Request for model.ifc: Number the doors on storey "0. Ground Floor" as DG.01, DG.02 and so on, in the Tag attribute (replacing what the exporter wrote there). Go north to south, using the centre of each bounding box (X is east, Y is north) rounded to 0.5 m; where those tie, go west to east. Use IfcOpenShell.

First a look at what the model holds.

```python
import ifcopenshell
import ifcopenshell.util.element
import ifcopenshell.util.placement

model = ifcopenshell.open("model.ifc")
print(model.schema)
storey = next(s for s in model.by_type("IfcBuildingStorey") if s.Name == "0. Ground Floor")
doors = [e for e in ifcopenshell.util.element.get_decomposition(storey) if e.is_a("IfcDoor")]
for e in sorted(doors, key=lambda e: e.id()):
    origin = ifcopenshell.util.placement.get_local_placement(e.ObjectPlacement)[:3, 3]
    print(e.id(), e.Tag, e.Name, origin.round(2) + 0.0, sep=" | ")
```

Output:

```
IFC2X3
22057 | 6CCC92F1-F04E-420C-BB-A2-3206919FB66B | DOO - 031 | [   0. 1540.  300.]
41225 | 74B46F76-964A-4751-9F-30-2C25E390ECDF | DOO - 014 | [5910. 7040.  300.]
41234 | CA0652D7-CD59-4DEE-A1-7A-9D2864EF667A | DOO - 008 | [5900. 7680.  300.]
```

```python
import ifcopenshell
import ifcopenshell.geom
import ifcopenshell.util.element
import ifcopenshell.util.shape

model = ifcopenshell.open("model.ifc")
settings = ifcopenshell.geom.settings()
settings.set("use-world-coords", True)


def centre(element):
    shape = ifcopenshell.geom.create_shape(settings, element)
    return ifcopenshell.util.shape.get_bbox_centroid(shape.geometry)


storey = next(s for s in model.by_type("IfcBuildingStorey") if s.Name == "0. Ground Floor")
doors = [e for e in ifcopenshell.util.element.get_decomposition(storey) if e.is_a("IfcDoor")]

# Insertion points can sit at a corner or the storey origin, so sort by the geometry (in metres).
centres = {e: centre(e) for e in doors}
doors.sort(key=lambda e: (-round(centres[e][1] / 0.5), centres[e][0]))

for i, e in enumerate(doors, start=1):
    number = f"DG.{i:02d}"
    e.Tag = number
    print(e.id(), number)

model.write("model-out.ifc")
```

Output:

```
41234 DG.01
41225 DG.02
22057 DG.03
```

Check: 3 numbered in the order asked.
